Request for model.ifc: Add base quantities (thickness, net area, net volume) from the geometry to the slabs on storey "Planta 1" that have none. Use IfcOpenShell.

First a look at what the model holds.

```python
import ifcopenshell
import ifcopenshell.util.element
import ifcopenshell.util.unit

model = ifcopenshell.open("model.ifc")
print(model.schema)
for unit_type in ("LENGTHUNIT", "AREAUNIT", "VOLUMEUNIT"):
    print(unit_type, ifcopenshell.util.unit.calculate_unit_scale(model, unit_type))
storey = next(s for s in model.by_type("IfcBuildingStorey") if s.Name == "Planta 1")
slabs = [e for e in ifcopenshell.util.element.get_decomposition(storey) if e.is_a("IfcSlab")]
for e in sorted(slabs, key=lambda e: e.id()):
    print(e.id(), e.is_a(), e.Name, list(ifcopenshell.util.element.get_psets(e, qtos_only=True)), sep=" | ")
```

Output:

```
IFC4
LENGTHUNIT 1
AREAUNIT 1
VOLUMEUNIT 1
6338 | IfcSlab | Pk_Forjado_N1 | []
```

```python
import ifcopenshell
import ifcopenshell.api.pset
import ifcopenshell.geom
import ifcopenshell.util.element
import ifcopenshell.util.shape
import ifcopenshell.util.unit

model = ifcopenshell.open("model.ifc")
unit_scale = ifcopenshell.util.unit.calculate_unit_scale(model)
area_scale = ifcopenshell.util.unit.calculate_unit_scale(model, "AREAUNIT")
volume_scale = ifcopenshell.util.unit.calculate_unit_scale(model, "VOLUMEUNIT")
settings = ifcopenshell.geom.settings()

storey = next(s for s in model.by_type("IfcBuildingStorey") if s.Name == "Planta 1")
slabs = [e for e in ifcopenshell.util.element.get_decomposition(storey) if e.is_a("IfcSlab")]

for e in sorted(slabs, key=lambda e: e.id()):
    if ifcopenshell.util.element.get_psets(e, qtos_only=True, should_inherit=False):
        continue
    # Geometry comes back in metres, in the element's own axes.
    shape = ifcopenshell.geom.create_shape(settings, e)
    values = {
        "Width": ifcopenshell.util.shape.get_z(shape.geometry) / unit_scale,
        "NetArea": ifcopenshell.util.shape.get_footprint_area(shape.geometry) / area_scale,
        "NetVolume": ifcopenshell.util.shape.get_volume(shape.geometry) / volume_scale,
    }
    qto = ifcopenshell.api.pset.add_qto(model, product=e, name="Qto_SlabBaseQuantities")
    ifcopenshell.api.pset.edit_qto(model, qto=qto, properties=values)
    print(e.id(), {k: round(v, 3) for k, v in values.items()})

model.write("model_rev.ifc")
```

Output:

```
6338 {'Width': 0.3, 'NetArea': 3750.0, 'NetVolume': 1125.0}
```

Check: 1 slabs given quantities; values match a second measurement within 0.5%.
